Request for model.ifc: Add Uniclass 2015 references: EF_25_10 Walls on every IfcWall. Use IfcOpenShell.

First a look at what the model holds.

```python
import ifcopenshell

model = ifcopenshell.open("model.ifc")
print(model.schema)
print("classifications:", [c.Name for c in model.by_type("IfcClassification")])
for ifc_class in ("IfcDoor", "IfcRoof", "IfcStair", "IfcWall", "IfcWindow"):
    print(ifc_class, len(model.by_type(ifc_class)))
```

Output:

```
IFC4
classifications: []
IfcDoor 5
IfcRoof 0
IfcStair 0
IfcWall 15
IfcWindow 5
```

```python
import ifcopenshell
import ifcopenshell.api.classification

model = ifcopenshell.open("model.ifc")

system = ifcopenshell.api.classification.add_classification(model, classification="Uniclass 2015")

codes = {
    "IfcWall": ("EF_25_10", "Walls"),
}
for ifc_class, (code, name) in codes.items():
    products = model.by_type(ifc_class)
    ifcopenshell.api.classification.add_reference(
        model, products=products, classification=system, identification=code, name=name
    )
    print(code, len(products))

model.write("model-out.ifc")
```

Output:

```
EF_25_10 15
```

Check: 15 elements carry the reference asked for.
